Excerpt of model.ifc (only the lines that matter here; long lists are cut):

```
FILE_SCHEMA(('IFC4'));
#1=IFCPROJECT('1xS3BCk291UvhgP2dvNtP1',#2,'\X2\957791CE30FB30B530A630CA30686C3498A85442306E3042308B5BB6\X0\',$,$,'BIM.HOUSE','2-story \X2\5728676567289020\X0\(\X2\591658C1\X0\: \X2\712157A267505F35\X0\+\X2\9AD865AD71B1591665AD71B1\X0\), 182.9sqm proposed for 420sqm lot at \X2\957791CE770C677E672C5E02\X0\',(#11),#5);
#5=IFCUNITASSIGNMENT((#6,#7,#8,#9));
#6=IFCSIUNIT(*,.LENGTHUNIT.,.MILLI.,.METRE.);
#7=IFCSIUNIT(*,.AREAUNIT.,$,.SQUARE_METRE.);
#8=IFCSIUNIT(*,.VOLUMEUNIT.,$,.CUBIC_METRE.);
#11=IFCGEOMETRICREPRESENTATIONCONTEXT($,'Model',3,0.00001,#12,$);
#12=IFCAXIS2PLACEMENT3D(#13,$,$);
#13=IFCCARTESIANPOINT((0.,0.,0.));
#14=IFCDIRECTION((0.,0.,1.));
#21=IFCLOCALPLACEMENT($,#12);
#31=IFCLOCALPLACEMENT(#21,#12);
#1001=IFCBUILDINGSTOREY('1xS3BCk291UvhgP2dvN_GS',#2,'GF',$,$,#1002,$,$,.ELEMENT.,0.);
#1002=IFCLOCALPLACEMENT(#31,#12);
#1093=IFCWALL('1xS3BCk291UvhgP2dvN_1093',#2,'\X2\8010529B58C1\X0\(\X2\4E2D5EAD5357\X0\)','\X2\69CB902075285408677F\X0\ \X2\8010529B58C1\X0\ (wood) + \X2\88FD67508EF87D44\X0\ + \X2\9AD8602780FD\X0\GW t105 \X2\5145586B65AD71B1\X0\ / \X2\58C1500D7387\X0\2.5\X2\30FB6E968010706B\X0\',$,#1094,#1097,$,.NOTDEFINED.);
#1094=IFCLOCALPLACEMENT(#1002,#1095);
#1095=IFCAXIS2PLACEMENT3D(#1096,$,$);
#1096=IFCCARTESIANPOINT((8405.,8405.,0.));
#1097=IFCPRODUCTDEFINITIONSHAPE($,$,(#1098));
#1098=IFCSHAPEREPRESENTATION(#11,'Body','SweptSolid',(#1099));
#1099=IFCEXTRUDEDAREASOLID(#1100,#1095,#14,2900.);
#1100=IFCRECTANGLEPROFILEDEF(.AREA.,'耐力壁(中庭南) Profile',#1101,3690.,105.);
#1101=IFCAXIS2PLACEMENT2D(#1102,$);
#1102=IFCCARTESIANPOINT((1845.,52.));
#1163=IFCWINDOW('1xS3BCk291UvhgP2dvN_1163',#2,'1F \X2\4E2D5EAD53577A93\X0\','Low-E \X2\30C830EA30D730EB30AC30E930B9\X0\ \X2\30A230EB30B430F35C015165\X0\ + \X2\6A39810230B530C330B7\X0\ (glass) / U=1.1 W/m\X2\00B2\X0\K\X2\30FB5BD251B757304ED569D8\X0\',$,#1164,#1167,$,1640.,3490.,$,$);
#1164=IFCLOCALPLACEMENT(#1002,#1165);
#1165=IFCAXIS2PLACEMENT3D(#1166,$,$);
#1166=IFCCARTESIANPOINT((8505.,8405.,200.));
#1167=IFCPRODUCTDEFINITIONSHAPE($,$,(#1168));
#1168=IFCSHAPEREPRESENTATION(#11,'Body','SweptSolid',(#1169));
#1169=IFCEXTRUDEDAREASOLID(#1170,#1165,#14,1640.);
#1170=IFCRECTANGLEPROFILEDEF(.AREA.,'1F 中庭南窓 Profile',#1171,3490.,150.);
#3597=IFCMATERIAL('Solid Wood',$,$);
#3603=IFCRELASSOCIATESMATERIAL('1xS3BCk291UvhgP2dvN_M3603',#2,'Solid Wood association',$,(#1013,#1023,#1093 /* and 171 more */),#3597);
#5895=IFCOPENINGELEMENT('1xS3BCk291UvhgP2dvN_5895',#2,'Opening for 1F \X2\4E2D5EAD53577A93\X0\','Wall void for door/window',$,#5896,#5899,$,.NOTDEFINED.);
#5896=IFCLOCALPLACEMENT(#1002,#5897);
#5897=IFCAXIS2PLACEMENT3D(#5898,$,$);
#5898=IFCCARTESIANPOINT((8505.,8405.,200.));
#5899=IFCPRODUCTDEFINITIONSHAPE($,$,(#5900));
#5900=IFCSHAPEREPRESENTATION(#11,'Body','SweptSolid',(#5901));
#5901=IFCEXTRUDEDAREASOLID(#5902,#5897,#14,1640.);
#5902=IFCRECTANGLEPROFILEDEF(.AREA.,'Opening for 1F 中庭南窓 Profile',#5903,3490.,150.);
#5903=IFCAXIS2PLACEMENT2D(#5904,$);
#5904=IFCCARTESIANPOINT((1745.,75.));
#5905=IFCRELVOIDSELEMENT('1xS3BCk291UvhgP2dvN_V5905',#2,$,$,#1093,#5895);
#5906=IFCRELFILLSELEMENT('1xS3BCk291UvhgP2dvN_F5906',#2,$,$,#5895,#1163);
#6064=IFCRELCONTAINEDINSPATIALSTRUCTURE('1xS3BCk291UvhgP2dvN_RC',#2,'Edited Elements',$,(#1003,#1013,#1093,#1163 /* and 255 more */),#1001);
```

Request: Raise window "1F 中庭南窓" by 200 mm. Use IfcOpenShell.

```python
import numpy as np
import ifcopenshell
import ifcopenshell.api.geometry
import ifcopenshell.util.placement
import ifcopenshell.util.unit

model = ifcopenshell.open("model.ifc")
unit_scale = ifcopenshell.util.unit.calculate_unit_scale(model)

window = model.by_guid("1xS3BCk291UvhgP2dvN_1163")
opening = window.FillsVoids[0].RelatingOpeningElement
dz = 200.0

shift = np.array([0.0, 0.0, dz])
# The window is not placed relative to its opening, so move both.
for product in (opening, window):
    matrix = ifcopenshell.util.placement.get_local_placement(product.ObjectPlacement)
    matrix[:3, 3] += shift
    ifcopenshell.api.geometry.edit_object_placement(model, product=product, matrix=matrix, is_si=False)

print(f"moved by {dz * unit_scale:+.3f} m")

model.write("model_edited.ifc")
```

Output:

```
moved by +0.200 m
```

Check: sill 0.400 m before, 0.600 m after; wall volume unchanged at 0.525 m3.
